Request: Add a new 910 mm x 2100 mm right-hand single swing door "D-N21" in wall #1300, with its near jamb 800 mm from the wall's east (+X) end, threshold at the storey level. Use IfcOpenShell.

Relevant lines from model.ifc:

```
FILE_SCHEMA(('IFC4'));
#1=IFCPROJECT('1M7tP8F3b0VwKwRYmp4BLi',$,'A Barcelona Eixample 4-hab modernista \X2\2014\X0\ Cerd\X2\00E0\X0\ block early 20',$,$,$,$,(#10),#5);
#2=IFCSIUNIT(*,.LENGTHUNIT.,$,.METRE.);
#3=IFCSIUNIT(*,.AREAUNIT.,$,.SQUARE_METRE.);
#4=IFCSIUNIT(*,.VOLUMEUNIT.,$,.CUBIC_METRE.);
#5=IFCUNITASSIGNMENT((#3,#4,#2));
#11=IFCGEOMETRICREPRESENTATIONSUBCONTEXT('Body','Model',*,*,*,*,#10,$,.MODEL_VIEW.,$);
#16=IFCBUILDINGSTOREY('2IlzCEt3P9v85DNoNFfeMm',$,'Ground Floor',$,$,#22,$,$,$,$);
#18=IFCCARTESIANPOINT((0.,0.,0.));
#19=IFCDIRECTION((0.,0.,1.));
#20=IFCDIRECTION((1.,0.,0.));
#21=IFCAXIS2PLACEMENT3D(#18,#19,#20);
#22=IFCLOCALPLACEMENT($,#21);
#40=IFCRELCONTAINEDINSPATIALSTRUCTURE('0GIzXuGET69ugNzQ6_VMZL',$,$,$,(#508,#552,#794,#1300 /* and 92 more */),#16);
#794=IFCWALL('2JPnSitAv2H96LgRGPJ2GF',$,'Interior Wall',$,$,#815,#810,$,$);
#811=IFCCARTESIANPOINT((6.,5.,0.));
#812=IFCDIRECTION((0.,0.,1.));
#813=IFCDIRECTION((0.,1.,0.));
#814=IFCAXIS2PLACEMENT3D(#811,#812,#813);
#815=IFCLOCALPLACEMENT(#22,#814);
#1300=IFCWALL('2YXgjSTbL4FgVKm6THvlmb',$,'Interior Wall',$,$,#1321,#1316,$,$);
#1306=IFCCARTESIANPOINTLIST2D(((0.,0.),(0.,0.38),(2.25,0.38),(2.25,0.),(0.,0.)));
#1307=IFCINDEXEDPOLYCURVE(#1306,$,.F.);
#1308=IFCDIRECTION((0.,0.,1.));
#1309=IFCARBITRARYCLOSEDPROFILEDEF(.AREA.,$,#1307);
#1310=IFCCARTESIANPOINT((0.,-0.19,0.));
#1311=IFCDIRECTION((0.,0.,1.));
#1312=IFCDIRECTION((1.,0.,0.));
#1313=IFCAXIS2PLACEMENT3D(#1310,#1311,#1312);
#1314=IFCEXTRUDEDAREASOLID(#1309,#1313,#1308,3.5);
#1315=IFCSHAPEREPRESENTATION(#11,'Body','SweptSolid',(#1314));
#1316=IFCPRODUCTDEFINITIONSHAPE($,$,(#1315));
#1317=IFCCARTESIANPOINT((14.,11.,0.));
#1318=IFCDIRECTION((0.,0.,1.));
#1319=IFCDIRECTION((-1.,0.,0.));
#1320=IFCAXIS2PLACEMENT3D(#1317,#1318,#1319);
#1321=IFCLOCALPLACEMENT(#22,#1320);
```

```python
import numpy as np
import ifcopenshell
import ifcopenshell.api.feature
import ifcopenshell.api.geometry
import ifcopenshell.api.root
import ifcopenshell.api.spatial
import ifcopenshell.geom
import ifcopenshell.util.element
import ifcopenshell.util.placement
import ifcopenshell.util.representation
import ifcopenshell.util.shape
import ifcopenshell.util.unit

model = ifcopenshell.open("model.ifc")
unit_scale = ifcopenshell.util.unit.calculate_unit_scale(model)
settings = ifcopenshell.geom.settings()


def volume(element):
    """Net volume in cubic metres, openings subtracted."""
    shape = ifcopenshell.geom.create_shape(settings, element)
    return ifcopenshell.util.shape.get_volume(shape.geometry)


wall = model.by_guid("2YXgjSTbL4FgVKm6THvlmb")
storey = ifcopenshell.util.element.get_container(wall, ifc_class="IfcBuildingStorey")
context = ifcopenshell.util.representation.get_context(model, "Model", "Body", "MODEL_VIEW")
before = volume(wall)

width, height, from_end, sill = 0.91, 2.1, 0.8, 0.0  # metres

# The wall runs along its own X axis, and the end named is its -X end.
wall_shape = ifcopenshell.geom.create_shape(settings, wall)
x, y, z = ifcopenshell.util.shape.get_vertices(wall_shape.geometry).T
start = x.min() + from_end
face, thickness = float(y.min()), float(y.max() - y.min())
wall_matrix = ifcopenshell.util.placement.get_local_placement(wall.ObjectPlacement)
level = ifcopenshell.util.placement.get_local_placement(storey.ObjectPlacement)[2, 3]


def in_wall(x, y):
    """Placement at x, y metres in the wall's axes, at sill height."""
    matrix = wall_matrix.copy()
    matrix[:, 3] = wall_matrix @ np.array([x / unit_scale, y / unit_scale, 0.0, 1.0])
    matrix[2, 3] = level + sill / unit_scale
    return matrix


# Opening: a box that overshoots both wall faces by 50 mm.
opening = ifcopenshell.api.root.create_entity(model, ifc_class="IfcOpeningElement", predefined_type="OPENING")
box = ifcopenshell.api.geometry.add_wall_representation(
    model, context=context, length=width, height=height, thickness=thickness + 0.1
)
ifcopenshell.api.geometry.assign_representation(model, product=opening, representation=box)
ifcopenshell.api.geometry.edit_object_placement(model, product=opening, matrix=in_wall(start, face - 0.05), is_si=False)
ifcopenshell.api.feature.add_feature(model, feature=opening, element=wall)

door = ifcopenshell.api.root.create_entity(model, ifc_class="IfcDoor", name="D-N21", predefined_type="DOOR")
door.OverallWidth, door.OverallHeight = width / unit_scale, height / unit_scale
door.OperationType = "SINGLE_SWING_RIGHT"
body = ifcopenshell.api.geometry.add_door_representation(
    model,
    context=context,
    overall_width=door.OverallWidth,
    overall_height=door.OverallHeight,
    operation_type="SINGLE_SWING_RIGHT",
    lining_properties={"LiningDepth": thickness / unit_scale, "ThresholdDepth": thickness / unit_scale},
)
ifcopenshell.api.geometry.assign_representation(model, product=door, representation=body)
ifcopenshell.api.spatial.assign_container(model, products=[door], relating_structure=storey)
ifcopenshell.api.feature.add_filling(model, opening=opening, element=door)

# The lining spans the wall, so the door starts at the wall face.
ifcopenshell.api.geometry.edit_object_placement(model, product=door, matrix=in_wall(start, face), is_si=False)

after = volume(wall)

print(f"wall volume {before:.3f} -> {after:.3f} m3")

model.write("model_updated.ifc")
```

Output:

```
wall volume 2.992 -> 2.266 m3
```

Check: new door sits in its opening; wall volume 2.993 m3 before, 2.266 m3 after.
